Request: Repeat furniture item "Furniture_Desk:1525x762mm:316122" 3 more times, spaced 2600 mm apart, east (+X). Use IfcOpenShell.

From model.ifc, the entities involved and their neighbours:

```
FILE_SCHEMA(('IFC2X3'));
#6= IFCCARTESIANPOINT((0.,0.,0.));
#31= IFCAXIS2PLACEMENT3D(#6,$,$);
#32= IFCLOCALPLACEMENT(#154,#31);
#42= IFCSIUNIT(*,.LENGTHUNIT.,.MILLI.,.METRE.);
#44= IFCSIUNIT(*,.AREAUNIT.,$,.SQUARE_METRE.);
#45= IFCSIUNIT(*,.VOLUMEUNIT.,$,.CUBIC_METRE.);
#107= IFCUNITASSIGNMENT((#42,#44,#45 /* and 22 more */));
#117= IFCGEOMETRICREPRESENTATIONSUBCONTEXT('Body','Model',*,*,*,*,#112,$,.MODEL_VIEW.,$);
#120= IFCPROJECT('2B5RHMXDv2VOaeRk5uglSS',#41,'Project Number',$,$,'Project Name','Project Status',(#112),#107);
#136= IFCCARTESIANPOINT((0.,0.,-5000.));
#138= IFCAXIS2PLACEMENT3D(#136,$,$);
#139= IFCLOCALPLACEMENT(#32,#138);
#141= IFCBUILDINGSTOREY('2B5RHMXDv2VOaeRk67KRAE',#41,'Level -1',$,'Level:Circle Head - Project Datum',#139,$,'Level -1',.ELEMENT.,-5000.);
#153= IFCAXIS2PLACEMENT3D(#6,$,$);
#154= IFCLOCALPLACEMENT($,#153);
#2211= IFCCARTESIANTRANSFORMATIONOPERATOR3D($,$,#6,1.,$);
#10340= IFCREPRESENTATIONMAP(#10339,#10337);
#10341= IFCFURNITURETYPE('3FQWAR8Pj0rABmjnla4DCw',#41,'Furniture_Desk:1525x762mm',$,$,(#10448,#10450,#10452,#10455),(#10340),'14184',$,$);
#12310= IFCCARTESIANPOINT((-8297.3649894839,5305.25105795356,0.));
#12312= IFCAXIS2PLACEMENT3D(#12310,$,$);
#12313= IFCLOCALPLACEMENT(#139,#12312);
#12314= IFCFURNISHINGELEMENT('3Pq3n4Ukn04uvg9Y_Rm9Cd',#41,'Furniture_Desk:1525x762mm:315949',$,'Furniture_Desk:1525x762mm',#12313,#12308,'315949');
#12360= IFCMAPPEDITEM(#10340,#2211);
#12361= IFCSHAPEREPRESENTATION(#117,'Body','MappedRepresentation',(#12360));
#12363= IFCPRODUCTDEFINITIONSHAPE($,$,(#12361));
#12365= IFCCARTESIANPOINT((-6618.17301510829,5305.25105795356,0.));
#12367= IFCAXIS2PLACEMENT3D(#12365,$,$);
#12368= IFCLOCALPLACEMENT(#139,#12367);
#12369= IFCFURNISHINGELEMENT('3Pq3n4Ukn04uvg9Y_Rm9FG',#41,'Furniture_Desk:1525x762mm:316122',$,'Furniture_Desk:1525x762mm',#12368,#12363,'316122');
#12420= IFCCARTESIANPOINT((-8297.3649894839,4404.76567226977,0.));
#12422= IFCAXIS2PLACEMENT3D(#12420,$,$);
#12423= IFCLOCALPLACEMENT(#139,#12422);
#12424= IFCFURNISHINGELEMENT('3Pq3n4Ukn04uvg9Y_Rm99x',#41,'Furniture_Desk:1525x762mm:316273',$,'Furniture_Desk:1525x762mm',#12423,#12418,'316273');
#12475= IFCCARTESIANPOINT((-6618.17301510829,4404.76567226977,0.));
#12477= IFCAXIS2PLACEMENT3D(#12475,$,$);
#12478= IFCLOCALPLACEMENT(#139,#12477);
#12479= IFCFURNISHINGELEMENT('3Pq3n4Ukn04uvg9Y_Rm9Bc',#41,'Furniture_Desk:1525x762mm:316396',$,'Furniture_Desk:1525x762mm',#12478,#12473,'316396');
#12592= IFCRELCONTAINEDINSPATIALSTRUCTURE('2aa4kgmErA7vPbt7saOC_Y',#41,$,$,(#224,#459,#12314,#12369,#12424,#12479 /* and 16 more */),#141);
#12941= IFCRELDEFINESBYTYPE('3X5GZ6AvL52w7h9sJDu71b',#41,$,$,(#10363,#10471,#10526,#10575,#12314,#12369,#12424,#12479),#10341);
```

```python
import numpy as np
import ifcopenshell
import ifcopenshell.api.geometry
import ifcopenshell.api.root
import ifcopenshell.util.element
import ifcopenshell.util.placement

model = ifcopenshell.open("model.ifc")


def reuse_history(source, copy):
    """copy_class also copies each property set's owner history, people and application; keep the originals."""
    for rel in copy.IsDefinedBy:
        if rel.is_a("IfcRelDefinesByProperties") and (history := rel.RelatingPropertyDefinition.OwnerHistory):
            rel.RelatingPropertyDefinition.OwnerHistory = source.OwnerHistory
            ifcopenshell.util.element.remove_deep2(model, history)


source = model.by_guid("3Pq3n4Ukn04uvg9Y_Rm9FG")
base = ifcopenshell.util.placement.get_local_placement(source.ObjectPlacement)
step = np.array([1.0, 0.0, 0.0]) * 2600.0

for i in range(1, 4):
    copy = ifcopenshell.api.root.copy_class(model, product=source)
    copy.Representation = ifcopenshell.util.element.copy_deep(
        model, source.Representation, exclude=["IfcGeometricRepresentationContext", "IfcRepresentationMap"]
    )
    copy.Name = "Furniture_Desk:1525x762mm"
    copy.Tag = None
    reuse_history(source, copy)
    matrix = base.copy()
    matrix[:3, 3] += i * step
    print("added at", matrix[:3, 3].round(3) + 0.0)
    ifcopenshell.api.geometry.edit_object_placement(model, product=copy, matrix=matrix, is_si=False)

model.write("model_updated.ifc")
```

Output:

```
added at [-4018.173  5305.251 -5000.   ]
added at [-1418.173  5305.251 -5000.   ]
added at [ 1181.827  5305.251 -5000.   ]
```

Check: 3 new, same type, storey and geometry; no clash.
